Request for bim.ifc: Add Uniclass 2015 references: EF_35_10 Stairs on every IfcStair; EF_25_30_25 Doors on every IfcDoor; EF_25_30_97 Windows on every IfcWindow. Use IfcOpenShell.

First a look at what the model holds.

```python
import ifcopenshell

model = ifcopenshell.open("bim.ifc")
print(model.schema)
print("classifications:", [c.Name for c in model.by_type("IfcClassification")])
for ifc_class in ("IfcDoor", "IfcRoof", "IfcStair", "IfcWall", "IfcWindow"):
    print(ifc_class, len(model.by_type(ifc_class)))
```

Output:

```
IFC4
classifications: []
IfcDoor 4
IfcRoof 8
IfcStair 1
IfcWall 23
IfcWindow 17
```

```python
import ifcopenshell
import ifcopenshell.api.classification

model = ifcopenshell.open("bim.ifc")

system = ifcopenshell.api.classification.add_classification(model, classification="Uniclass 2015")

codes = {
    "IfcStair": ("EF_35_10", "Stairs"),
    "IfcDoor": ("EF_25_30_25", "Doors"),
    "IfcWindow": ("EF_25_30_97", "Windows"),
}
for ifc_class, (code, name) in codes.items():
    products = model.by_type(ifc_class)
    ifcopenshell.api.classification.add_reference(
        model, products=products, classification=system, identification=code, name=name
    )
    print(code, len(products))

model.write("bim_v2.ifc")
```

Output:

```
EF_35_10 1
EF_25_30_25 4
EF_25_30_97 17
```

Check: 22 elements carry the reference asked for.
